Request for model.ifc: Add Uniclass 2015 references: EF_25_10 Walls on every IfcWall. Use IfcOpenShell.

First a look at what the model holds.

```python
import ifcopenshell

model = ifcopenshell.open("model.ifc")
print(model.schema)
print("classifications:", [c.Name for c in model.by_type("IfcClassification")])
for ifc_class in ("IfcDoor", "IfcRoof", "IfcStair", "IfcWall", "IfcWindow"):
    print(ifc_class, len(model.by_type(ifc_class)))
```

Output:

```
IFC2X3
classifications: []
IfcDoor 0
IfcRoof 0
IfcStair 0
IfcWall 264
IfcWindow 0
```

```python
import ifcopenshell
import ifcopenshell.api.classification

model = ifcopenshell.open("model.ifc")

# IFC2X3 requires Source and Edition and has no link from the project to the system.
system = model.create_entity("IfcClassification", Source="NBS", Edition="2015", Name="Uniclass 2015")

codes = {
    "IfcWall": ("EF_25_10", "Walls"),
}
for ifc_class, (code, name) in codes.items():
    products = model.by_type(ifc_class)
    ifcopenshell.api.classification.add_reference(
        model, products=products, classification=system, identification=code, name=name
    )
    print(code, len(products))

model.write("model_rev.ifc")
```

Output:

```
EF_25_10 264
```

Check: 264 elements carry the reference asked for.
